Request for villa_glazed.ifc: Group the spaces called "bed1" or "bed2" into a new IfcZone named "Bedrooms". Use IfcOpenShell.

First a look at what the model holds.

```python
import ifcopenshell

model = ifcopenshell.open("villa_glazed.ifc")
print(model.schema)
seen = {}
for space in model.by_type("IfcSpace"):
    seen[space.LongName] = seen.get(space.LongName, 0) + 1
for name, count in sorted(seen.items(), key=str):
    print(count, "x", name)
print("zones:", [z.Name for z in model.by_type("IfcZone")][:20])
```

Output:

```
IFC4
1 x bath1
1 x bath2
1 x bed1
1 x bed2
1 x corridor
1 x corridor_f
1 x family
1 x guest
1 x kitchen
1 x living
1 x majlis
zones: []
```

```python
import ifcopenshell
import ifcopenshell.api.group
import ifcopenshell.api.root

model = ifcopenshell.open("villa_glazed.ifc")

names = {"bed1", "bed2"}
spaces = [s for s in model.by_type("IfcSpace") if s.LongName in names]

zone = ifcopenshell.api.root.create_entity(model, ifc_class="IfcZone", name="Bedrooms")
ifcopenshell.api.group.assign_group(model, products=spaces, group=zone)
print(len(spaces), "spaces in", zone.Name)

model.write("villa_glazed_v2.ifc")
```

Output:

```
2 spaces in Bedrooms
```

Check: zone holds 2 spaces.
